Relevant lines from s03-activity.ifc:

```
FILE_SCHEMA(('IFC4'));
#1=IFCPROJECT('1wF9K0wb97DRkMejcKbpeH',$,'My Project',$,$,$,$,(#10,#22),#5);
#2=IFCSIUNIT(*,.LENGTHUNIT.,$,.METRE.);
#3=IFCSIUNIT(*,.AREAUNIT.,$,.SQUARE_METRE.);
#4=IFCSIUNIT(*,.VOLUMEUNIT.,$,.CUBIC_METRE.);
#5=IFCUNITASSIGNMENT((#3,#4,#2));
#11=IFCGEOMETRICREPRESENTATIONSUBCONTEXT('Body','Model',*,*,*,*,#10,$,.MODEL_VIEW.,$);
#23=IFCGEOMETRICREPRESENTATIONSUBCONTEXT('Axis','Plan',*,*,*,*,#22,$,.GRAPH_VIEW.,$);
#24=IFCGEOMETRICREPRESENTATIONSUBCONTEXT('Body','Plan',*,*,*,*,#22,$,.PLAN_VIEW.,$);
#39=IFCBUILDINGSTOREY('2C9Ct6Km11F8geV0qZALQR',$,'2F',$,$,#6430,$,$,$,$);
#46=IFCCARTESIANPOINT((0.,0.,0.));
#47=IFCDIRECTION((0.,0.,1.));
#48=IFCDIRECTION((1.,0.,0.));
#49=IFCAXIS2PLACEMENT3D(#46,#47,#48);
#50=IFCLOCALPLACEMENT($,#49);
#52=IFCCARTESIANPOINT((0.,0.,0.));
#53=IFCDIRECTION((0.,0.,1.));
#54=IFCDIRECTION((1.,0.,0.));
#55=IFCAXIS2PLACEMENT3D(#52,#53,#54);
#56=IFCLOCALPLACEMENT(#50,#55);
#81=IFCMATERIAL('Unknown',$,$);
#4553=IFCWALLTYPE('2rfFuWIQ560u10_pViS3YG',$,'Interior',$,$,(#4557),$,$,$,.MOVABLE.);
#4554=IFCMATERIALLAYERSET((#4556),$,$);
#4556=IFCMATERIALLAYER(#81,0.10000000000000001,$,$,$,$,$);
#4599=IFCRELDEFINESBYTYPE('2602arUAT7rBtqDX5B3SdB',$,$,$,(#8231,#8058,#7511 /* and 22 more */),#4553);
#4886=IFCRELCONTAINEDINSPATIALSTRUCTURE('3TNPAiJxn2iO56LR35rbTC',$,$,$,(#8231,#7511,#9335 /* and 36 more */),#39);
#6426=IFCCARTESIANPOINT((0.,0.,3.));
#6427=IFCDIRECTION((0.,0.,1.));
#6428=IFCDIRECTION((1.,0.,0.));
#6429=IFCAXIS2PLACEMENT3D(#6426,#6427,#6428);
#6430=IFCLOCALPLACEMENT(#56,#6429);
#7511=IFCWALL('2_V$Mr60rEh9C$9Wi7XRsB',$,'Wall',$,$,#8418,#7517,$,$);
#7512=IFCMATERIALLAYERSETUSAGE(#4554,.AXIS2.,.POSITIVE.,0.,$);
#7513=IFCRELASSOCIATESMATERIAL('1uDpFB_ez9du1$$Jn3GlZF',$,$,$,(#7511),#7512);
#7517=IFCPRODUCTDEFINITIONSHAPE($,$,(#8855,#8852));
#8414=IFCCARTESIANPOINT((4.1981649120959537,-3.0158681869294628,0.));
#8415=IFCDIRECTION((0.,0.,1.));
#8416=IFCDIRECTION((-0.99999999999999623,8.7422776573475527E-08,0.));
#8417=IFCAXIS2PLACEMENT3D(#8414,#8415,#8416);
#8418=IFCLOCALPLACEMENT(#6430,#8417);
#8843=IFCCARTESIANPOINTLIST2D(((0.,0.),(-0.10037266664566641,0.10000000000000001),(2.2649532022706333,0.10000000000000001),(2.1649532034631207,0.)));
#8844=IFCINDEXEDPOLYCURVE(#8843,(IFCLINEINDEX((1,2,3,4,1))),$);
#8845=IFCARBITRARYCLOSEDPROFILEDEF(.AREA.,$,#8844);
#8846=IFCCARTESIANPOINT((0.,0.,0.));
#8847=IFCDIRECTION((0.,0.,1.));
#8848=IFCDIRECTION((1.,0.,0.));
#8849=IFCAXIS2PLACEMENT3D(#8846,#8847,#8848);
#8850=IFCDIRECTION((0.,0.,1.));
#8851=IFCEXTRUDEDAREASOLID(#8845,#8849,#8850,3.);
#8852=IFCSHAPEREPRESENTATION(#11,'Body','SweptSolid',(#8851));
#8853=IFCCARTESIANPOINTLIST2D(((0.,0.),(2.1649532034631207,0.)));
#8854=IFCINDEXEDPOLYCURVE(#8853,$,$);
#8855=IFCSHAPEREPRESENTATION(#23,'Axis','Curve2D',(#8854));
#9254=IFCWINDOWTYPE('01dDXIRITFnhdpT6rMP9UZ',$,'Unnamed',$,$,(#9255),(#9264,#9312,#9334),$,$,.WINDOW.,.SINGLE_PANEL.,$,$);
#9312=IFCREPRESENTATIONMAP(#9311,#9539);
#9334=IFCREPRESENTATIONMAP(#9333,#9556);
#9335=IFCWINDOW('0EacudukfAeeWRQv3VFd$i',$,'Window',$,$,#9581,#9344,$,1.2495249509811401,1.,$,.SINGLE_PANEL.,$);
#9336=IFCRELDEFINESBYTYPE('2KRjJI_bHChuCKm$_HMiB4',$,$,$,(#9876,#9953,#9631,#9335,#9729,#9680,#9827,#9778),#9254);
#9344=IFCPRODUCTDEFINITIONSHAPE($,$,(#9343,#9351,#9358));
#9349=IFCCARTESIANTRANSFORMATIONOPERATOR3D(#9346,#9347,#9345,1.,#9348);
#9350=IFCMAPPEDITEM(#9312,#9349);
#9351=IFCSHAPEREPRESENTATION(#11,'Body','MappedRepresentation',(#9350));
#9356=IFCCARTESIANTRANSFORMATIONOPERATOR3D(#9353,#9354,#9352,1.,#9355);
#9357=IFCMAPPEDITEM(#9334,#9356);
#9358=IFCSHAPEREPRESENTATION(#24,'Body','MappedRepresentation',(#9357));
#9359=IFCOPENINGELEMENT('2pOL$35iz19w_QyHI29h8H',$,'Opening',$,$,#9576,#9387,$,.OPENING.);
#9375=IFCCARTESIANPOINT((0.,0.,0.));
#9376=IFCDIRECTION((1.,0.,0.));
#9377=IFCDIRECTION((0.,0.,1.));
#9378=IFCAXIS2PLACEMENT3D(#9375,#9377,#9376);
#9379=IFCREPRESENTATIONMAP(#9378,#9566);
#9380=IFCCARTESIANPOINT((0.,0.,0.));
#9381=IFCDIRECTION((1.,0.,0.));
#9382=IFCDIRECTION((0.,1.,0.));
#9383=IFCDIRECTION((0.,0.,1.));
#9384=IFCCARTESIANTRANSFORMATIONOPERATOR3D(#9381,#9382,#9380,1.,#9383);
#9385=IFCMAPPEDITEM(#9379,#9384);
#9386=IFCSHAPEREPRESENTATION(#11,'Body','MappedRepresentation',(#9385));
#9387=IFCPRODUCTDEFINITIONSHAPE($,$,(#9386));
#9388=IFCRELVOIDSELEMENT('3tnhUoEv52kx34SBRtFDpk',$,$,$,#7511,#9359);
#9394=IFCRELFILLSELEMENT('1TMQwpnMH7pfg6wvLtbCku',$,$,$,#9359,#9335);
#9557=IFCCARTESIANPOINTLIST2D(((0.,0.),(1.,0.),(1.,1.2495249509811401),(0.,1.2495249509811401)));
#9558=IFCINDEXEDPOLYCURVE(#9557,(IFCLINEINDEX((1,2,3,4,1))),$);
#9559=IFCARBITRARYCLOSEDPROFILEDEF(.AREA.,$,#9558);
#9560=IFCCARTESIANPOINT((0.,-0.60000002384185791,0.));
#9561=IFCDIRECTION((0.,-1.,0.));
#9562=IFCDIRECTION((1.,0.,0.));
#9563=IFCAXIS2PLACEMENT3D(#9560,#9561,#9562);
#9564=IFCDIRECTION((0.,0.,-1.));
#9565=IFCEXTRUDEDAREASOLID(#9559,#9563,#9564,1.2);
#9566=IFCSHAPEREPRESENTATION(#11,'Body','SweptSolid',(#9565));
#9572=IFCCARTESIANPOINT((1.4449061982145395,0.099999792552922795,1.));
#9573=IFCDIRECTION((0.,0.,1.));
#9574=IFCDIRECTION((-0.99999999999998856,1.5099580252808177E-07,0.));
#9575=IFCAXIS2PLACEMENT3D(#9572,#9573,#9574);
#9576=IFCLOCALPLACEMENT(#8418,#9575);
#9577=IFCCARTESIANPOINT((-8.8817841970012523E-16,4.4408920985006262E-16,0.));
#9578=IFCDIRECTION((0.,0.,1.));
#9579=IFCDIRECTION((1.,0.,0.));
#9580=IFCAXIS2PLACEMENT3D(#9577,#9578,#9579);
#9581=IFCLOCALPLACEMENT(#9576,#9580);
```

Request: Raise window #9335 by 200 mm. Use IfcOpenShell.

```python
import numpy as np
import ifcopenshell
import ifcopenshell.api.geometry
import ifcopenshell.util.placement
import ifcopenshell.util.unit

model = ifcopenshell.open("s03-activity.ifc")
unit_scale = ifcopenshell.util.unit.calculate_unit_scale(model)

window = model.by_id(9335)
opening = window.FillsVoids[0].RelatingOpeningElement
dz = 0.2 / unit_scale

shift = np.array([0.0, 0.0, dz])
# The window is placed relative to its opening, so it follows when the opening moves.
matrix = ifcopenshell.util.placement.get_local_placement(opening.ObjectPlacement)
matrix[:3, 3] += shift
ifcopenshell.api.geometry.edit_object_placement(
    model, product=opening, matrix=matrix, is_si=False, should_transform_children=True
)

print(f"moved by {dz * unit_scale:+.3f} m")

model.write("s03-activity_edited.ifc")
```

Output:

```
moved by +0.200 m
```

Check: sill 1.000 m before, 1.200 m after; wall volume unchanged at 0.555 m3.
